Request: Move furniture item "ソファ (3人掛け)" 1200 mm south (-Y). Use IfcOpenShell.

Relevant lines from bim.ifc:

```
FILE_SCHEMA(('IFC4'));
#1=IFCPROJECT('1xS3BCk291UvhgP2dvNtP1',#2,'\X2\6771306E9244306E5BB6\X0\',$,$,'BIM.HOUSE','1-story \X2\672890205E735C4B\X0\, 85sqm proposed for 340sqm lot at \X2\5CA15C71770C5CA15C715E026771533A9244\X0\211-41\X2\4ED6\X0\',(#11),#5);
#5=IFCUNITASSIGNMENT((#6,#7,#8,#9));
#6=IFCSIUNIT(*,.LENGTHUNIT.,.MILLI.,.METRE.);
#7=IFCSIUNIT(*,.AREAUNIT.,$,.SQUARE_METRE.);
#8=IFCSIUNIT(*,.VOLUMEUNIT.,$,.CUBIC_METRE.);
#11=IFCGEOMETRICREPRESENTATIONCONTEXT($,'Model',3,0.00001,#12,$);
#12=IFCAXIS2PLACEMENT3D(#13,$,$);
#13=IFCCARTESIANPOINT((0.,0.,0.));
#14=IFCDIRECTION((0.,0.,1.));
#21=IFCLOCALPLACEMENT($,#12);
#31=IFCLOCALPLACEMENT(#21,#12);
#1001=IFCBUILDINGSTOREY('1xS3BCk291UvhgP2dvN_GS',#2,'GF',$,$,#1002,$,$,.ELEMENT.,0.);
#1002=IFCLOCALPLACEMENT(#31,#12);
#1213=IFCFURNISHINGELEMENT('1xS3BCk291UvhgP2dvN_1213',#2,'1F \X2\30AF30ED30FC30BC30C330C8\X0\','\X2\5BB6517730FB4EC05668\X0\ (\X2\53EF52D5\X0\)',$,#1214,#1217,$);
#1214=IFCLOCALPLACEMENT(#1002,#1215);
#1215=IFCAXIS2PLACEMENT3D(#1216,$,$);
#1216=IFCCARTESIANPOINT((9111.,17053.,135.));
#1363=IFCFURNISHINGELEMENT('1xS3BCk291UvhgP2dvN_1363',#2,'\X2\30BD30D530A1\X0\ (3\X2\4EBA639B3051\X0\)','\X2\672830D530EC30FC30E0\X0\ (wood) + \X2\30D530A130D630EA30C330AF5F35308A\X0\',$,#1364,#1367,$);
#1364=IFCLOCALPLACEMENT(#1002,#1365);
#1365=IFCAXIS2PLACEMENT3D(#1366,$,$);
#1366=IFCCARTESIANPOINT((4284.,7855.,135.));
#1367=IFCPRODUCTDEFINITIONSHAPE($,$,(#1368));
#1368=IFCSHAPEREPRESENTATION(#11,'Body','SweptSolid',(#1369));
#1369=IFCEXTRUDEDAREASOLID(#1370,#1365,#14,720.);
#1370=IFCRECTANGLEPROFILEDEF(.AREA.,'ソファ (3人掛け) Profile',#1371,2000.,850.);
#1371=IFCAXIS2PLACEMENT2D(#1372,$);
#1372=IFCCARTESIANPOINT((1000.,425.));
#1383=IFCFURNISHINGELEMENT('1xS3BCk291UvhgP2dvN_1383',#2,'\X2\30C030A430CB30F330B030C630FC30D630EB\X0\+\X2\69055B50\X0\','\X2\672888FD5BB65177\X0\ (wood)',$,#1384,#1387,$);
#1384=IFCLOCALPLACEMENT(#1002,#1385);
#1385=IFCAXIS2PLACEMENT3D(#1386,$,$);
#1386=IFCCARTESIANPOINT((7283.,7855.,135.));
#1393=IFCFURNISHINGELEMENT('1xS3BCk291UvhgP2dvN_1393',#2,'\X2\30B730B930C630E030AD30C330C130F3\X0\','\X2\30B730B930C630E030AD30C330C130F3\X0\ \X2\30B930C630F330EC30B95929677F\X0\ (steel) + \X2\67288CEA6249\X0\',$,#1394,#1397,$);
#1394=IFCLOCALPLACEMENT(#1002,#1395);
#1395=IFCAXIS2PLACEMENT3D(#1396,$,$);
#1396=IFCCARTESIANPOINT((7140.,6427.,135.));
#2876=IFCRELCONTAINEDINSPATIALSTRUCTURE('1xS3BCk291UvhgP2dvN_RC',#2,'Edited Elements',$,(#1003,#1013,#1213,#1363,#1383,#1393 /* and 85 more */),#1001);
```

```python
import ifcopenshell
import ifcopenshell.api.geometry
import ifcopenshell.util.placement
import ifcopenshell.util.unit

model = ifcopenshell.open("bim.ifc")
unit_scale = ifcopenshell.util.unit.calculate_unit_scale(model)

item = model.by_guid("1xS3BCk291UvhgP2dvN_1363")
matrix = ifcopenshell.util.placement.get_local_placement(item.ObjectPlacement)
matrix[1, 3] -= 1.2 / unit_scale
ifcopenshell.api.geometry.edit_object_placement(model, product=item, matrix=matrix, is_si=False)

print(ifcopenshell.util.placement.get_local_placement(item.ObjectPlacement).round(3) + 0.0)

model.write("bim_v2.ifc")
```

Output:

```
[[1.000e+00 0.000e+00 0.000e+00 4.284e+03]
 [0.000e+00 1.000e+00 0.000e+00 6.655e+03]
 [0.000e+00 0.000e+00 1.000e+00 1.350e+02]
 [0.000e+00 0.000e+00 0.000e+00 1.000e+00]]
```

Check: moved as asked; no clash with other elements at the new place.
